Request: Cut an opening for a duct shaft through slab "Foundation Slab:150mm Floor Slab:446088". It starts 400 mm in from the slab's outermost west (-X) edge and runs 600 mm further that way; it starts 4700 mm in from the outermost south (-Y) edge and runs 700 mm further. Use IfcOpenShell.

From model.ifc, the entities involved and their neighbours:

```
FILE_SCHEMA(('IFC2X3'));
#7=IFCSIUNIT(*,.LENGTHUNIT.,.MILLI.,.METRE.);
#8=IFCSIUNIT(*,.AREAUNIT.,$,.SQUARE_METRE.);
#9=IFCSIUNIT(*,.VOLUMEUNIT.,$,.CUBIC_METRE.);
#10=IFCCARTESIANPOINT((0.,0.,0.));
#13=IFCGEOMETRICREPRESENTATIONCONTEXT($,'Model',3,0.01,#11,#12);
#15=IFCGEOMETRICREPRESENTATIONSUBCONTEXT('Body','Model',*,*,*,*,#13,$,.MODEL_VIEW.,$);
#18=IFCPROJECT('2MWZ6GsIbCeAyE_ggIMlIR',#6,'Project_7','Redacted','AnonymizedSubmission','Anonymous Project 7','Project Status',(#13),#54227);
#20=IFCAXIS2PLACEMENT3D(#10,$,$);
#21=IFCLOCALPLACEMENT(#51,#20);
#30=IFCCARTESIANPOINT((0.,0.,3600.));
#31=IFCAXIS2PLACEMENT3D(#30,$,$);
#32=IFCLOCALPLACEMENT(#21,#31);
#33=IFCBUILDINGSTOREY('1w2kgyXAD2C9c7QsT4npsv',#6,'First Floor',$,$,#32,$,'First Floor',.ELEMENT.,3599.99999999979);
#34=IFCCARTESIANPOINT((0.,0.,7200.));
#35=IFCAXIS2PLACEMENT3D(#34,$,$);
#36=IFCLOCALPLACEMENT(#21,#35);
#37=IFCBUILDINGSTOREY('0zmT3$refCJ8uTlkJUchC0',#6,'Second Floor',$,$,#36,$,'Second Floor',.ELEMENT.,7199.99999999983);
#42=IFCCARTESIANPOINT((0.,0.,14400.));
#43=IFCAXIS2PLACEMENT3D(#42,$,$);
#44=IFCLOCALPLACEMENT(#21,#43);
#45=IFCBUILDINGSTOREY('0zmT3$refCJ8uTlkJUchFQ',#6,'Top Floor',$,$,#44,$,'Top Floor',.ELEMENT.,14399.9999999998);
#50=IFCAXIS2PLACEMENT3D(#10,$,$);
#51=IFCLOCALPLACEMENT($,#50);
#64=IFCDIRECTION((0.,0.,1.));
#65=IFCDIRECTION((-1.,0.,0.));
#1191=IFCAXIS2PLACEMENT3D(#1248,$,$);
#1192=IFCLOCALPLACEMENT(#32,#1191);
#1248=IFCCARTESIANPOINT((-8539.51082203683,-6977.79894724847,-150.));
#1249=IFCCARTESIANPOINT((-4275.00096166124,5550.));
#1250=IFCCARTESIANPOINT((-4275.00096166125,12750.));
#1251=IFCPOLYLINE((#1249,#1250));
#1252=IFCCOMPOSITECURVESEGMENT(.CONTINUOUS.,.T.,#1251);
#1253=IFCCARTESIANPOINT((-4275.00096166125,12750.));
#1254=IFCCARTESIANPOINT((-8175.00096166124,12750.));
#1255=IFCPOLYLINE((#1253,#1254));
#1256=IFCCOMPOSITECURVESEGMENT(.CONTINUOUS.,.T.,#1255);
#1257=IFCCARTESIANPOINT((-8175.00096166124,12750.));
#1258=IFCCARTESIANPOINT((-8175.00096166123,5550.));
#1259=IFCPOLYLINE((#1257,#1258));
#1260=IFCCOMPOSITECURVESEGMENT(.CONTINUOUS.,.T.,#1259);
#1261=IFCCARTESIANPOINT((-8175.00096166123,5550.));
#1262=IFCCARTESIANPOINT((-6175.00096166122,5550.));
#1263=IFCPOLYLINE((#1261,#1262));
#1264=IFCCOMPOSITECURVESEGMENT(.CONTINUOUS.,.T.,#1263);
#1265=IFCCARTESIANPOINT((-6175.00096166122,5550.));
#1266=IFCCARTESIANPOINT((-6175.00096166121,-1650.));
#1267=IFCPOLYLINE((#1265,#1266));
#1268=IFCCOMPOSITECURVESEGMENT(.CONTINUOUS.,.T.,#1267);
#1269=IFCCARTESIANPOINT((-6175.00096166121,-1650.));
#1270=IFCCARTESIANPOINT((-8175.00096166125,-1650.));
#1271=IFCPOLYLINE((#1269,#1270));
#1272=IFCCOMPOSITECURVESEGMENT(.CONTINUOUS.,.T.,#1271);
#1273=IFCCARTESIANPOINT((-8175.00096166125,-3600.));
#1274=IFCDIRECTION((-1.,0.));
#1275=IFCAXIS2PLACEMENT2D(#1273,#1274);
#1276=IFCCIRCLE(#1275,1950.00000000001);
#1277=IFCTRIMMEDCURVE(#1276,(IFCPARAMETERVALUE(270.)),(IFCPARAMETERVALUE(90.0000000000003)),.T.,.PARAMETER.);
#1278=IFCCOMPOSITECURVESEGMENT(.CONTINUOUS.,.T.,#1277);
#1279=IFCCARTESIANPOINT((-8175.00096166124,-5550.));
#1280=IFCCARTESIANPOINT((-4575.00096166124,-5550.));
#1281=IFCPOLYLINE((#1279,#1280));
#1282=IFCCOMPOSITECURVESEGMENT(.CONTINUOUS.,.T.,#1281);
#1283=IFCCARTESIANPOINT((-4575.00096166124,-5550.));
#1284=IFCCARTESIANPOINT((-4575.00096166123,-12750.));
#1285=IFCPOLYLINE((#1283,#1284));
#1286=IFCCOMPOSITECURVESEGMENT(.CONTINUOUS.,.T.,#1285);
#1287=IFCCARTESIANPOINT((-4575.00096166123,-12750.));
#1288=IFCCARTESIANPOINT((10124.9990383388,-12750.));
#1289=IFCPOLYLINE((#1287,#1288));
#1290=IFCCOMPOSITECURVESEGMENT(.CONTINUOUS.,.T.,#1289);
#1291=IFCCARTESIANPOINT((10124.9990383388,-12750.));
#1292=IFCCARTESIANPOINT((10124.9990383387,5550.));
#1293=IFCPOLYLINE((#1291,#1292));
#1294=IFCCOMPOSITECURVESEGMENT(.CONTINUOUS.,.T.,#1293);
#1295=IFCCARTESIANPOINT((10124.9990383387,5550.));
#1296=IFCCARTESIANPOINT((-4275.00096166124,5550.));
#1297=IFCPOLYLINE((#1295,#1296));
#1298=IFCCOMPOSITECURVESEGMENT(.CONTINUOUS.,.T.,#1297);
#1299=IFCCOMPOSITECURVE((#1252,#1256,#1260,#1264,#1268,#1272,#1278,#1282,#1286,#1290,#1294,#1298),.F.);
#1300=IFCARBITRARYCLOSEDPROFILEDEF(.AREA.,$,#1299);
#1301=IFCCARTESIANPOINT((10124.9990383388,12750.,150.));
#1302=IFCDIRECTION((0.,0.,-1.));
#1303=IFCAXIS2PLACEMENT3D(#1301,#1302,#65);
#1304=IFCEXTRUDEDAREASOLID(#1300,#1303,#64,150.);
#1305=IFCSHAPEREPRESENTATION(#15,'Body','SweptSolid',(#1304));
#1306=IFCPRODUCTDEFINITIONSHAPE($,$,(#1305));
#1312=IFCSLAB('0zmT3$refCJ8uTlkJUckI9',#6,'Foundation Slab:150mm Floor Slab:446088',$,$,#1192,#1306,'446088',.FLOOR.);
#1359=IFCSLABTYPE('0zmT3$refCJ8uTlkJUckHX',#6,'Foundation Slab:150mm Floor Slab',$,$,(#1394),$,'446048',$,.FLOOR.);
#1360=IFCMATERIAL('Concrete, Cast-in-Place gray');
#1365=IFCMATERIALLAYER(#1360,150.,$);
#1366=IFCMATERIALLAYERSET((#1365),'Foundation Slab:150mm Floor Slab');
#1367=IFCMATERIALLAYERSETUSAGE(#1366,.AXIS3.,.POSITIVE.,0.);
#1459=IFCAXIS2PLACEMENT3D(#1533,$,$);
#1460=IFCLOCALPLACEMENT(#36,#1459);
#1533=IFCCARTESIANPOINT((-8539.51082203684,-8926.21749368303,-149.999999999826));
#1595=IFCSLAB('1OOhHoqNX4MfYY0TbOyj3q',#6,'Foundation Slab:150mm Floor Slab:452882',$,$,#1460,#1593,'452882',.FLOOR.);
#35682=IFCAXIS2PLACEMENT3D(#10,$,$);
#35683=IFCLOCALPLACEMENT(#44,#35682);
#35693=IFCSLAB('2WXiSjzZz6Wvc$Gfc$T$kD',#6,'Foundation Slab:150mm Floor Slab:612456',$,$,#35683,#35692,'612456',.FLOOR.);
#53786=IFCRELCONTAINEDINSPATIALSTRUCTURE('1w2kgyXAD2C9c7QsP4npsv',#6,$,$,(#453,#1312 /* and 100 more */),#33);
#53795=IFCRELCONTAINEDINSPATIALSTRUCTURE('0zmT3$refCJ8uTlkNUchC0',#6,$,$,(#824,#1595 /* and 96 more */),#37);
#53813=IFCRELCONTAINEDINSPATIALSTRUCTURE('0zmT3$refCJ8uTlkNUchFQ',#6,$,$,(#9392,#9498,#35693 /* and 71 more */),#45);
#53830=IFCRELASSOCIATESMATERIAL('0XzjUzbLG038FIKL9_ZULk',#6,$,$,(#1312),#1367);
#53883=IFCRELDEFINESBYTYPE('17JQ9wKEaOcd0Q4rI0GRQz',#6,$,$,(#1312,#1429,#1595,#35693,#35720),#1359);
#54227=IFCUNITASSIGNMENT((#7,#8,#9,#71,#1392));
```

```python
import numpy as np
import ifcopenshell
import ifcopenshell.api.feature
import ifcopenshell.api.geometry
import ifcopenshell.api.root
import ifcopenshell.geom
import ifcopenshell.util.placement
import ifcopenshell.util.representation
import ifcopenshell.util.shape
import ifcopenshell.util.unit

model = ifcopenshell.open("model.ifc")
unit_scale = ifcopenshell.util.unit.calculate_unit_scale(model)
settings = ifcopenshell.geom.settings()


def volume(element):
    """Net volume in cubic metres, openings subtracted."""
    shape = ifcopenshell.geom.create_shape(settings, element)
    return ifcopenshell.util.shape.get_volume(shape.geometry)


slab = model.by_guid("0zmT3$refCJ8uTlkJUckI9")
before = volume(slab)

# Extent in the slab's own axes, in metres. The edges named are its -X and -Y sides.
slab_shape = ifcopenshell.geom.create_shape(settings, slab)
vertices = ifcopenshell.util.shape.get_vertices(slab_shape.geometry)
x_min, y_min, bottom = vertices.min(axis=0)
top = vertices[:, 2].max()

opening = ifcopenshell.api.root.create_entity(model, ifc_class="IfcOpeningElement", name="Duct shaft opening")
context = ifcopenshell.util.representation.get_context(model, "Model", "Body", "MODEL_VIEW")
width, depth = 0.6, 0.7
outline = [(0.0, 0.0), (width, 0.0), (width, depth), (0.0, depth), (0.0, 0.0)]
# Overshoot both faces by 50 mm so the cut is clean.
shape = ifcopenshell.api.geometry.add_slab_representation(
    model, context=context, depth=top - bottom + 0.1, polyline=outline
)
ifcopenshell.api.geometry.assign_representation(model, product=opening, representation=shape)

matrix = ifcopenshell.util.placement.get_local_placement(slab.ObjectPlacement)
matrix[:, 3] = matrix @ np.append(np.array([x_min + 0.4, y_min + 4.7, bottom - 0.05]) / unit_scale, 1.0)
ifcopenshell.api.geometry.edit_object_placement(model, product=opening, matrix=matrix, is_si=False)
ifcopenshell.api.feature.add_feature(model, feature=opening, element=slab)

after = volume(slab)

print(f"slab volume {before:.3f} -> {after:.3f} m3")

model.write("model-out.ifc")
```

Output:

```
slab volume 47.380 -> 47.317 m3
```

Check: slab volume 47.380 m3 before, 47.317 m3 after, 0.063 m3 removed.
